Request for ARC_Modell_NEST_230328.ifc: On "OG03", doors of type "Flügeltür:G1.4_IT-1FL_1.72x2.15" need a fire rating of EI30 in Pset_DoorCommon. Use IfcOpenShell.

First a look at what the model holds.

```python
import ifcopenshell
import ifcopenshell.util.element

model = ifcopenshell.open("ARC_Modell_NEST_230328.ifc")
print(model.schema)
storey = next(s for s in model.by_type("IfcBuildingStorey") if s.Name == "OG03")
doors = [e for e in ifcopenshell.util.element.get_decomposition(storey) if e.is_a("IfcDoor")]
seen = {}
for e in doors:
    element_type = ifcopenshell.util.element.get_type(e)
    key = (element_type.Name if element_type != e and element_type else None, ifcopenshell.util.element.get_pset(e, "Pset_DoorCommon", "FireRating"))
    seen[key] = seen.get(key, 0) + 1
for (name, value), count in sorted(seen.items(), key=str):
    print(count, "x", name, "|", value)
```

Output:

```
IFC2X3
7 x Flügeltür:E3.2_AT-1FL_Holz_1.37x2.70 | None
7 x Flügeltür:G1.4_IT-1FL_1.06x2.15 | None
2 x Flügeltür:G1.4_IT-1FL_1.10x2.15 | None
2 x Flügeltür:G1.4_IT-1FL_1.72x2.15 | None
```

```python
import ifcopenshell
import ifcopenshell.api.pset
import ifcopenshell.util.element

model = ifcopenshell.open("ARC_Modell_NEST_230328.ifc")

storey = next(s for s in model.by_type("IfcBuildingStorey") if s.Name == "OG03")
doors = [e for e in ifcopenshell.util.element.get_decomposition(storey) if e.is_a("IfcDoor")]

count = 0
for e in doors:
    element_type = ifcopenshell.util.element.get_type(e)
    if element_type in (None, e) or element_type.Name != "Flügeltür:G1.4_IT-1FL_1.72x2.15":
        continue
    # add_pset returns the element's existing set when there is one.
    pset = ifcopenshell.api.pset.add_pset(model, product=e, name="Pset_DoorCommon")
    ifcopenshell.api.pset.edit_pset(model, pset=pset, properties={"FireRating": "EI30"})
    count += 1

print(count, "doors updated")

model.write("ARC_Modell_NEST_230328_v2.ifc")
```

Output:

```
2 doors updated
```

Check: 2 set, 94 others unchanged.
